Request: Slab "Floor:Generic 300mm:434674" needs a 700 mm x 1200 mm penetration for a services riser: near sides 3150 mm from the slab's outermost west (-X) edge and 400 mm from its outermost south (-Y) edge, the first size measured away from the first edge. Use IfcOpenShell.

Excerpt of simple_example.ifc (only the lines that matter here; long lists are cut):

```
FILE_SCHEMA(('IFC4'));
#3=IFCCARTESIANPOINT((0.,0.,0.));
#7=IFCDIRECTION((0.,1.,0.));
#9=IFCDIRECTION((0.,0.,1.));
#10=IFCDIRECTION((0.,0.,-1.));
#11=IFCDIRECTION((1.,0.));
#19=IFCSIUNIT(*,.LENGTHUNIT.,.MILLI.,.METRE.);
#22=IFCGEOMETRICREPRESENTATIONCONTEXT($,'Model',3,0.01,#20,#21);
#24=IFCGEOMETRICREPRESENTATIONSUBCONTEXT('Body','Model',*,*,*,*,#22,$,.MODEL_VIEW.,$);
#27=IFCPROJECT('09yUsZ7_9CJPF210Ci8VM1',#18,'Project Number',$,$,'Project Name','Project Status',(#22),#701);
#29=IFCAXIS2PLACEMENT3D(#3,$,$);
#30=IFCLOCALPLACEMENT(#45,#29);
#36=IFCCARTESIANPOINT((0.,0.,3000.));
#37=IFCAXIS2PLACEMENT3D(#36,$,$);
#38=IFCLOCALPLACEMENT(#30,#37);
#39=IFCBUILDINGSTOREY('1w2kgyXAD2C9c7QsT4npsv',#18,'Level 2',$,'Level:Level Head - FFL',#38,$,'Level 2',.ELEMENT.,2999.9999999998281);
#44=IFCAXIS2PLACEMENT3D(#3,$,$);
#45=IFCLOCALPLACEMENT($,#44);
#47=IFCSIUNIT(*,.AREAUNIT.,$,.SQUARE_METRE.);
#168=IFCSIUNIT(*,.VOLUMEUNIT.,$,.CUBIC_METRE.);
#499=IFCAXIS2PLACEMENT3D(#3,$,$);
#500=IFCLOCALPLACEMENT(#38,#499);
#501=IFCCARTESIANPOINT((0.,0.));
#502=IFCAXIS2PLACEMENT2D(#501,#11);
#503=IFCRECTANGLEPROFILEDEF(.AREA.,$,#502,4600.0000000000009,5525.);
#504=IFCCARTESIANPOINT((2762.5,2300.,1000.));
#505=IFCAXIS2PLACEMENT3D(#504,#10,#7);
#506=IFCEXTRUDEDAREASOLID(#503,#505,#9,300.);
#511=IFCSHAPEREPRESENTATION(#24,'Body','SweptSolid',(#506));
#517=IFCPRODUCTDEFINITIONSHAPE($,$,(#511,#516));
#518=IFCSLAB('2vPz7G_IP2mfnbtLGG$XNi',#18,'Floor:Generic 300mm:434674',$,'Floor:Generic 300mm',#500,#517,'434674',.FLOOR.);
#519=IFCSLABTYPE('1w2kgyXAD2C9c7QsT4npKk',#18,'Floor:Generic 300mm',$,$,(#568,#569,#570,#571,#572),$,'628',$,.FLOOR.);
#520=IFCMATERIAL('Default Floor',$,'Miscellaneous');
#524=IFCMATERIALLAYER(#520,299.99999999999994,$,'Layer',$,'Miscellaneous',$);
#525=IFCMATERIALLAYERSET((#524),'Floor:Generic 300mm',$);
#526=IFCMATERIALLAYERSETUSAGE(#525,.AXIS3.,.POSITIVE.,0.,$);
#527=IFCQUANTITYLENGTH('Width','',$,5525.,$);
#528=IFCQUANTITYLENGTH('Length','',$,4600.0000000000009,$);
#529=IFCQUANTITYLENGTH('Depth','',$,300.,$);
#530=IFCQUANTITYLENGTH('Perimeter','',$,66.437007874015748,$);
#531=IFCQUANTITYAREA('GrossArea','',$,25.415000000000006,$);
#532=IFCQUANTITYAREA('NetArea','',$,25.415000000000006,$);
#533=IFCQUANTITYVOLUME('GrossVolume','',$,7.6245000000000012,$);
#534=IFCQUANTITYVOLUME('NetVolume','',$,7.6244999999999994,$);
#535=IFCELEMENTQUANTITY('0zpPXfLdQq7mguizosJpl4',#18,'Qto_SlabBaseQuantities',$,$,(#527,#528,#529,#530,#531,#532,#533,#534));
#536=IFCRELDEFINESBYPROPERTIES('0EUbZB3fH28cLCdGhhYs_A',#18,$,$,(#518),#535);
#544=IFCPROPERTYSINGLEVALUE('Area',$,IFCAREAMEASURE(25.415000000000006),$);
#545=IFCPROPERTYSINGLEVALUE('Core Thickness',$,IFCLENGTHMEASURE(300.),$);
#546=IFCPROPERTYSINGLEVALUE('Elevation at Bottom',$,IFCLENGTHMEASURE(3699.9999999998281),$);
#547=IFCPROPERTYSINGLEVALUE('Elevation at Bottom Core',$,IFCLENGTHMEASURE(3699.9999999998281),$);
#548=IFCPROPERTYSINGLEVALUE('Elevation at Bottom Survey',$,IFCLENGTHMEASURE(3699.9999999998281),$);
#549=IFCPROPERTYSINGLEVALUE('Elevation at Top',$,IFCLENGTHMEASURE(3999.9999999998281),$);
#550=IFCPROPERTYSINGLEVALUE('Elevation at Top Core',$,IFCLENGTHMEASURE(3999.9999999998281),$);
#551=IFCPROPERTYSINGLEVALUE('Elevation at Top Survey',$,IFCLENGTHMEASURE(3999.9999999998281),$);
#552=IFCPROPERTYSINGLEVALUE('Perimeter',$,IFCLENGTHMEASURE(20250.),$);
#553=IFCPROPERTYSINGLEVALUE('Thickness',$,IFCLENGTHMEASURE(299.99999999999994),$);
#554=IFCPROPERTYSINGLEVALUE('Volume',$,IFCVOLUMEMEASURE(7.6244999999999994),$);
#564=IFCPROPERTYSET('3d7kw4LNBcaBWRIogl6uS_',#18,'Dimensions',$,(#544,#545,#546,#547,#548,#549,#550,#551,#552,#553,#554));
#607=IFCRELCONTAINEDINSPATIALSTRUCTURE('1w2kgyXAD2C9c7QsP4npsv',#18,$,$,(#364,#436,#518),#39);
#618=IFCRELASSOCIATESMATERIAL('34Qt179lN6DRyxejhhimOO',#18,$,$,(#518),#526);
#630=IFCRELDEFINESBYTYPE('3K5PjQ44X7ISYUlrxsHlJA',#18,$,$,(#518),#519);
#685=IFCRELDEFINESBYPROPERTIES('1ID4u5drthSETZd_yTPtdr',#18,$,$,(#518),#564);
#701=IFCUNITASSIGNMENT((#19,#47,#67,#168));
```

```python
import numpy as np
import ifcopenshell
import ifcopenshell.api.feature
import ifcopenshell.api.geometry
import ifcopenshell.api.pset
import ifcopenshell.api.root
import ifcopenshell.geom
import ifcopenshell.util.element
import ifcopenshell.util.placement
import ifcopenshell.util.representation
import ifcopenshell.util.shape
import ifcopenshell.util.unit

model = ifcopenshell.open("simple_example.ifc")
unit_scale = ifcopenshell.util.unit.calculate_unit_scale(model)
area_scale = ifcopenshell.util.unit.calculate_unit_scale(model, "AREAUNIT")
volume_scale = ifcopenshell.util.unit.calculate_unit_scale(model, "VOLUMEUNIT")
settings = ifcopenshell.geom.settings()


def volume(element):
    """Net volume in cubic metres, openings subtracted."""
    shape = ifcopenshell.geom.create_shape(settings, element)
    return ifcopenshell.util.shape.get_volume(shape.geometry)


slab = model.by_id(518)
before = volume(slab)

# Extent in the slab's own axes, in metres. The edges named are its -X and -Y sides.
slab_shape = ifcopenshell.geom.create_shape(settings, slab)
vertices = ifcopenshell.util.shape.get_vertices(slab_shape.geometry)
x_min, y_min, bottom = vertices.min(axis=0)
top = vertices[:, 2].max()

opening = ifcopenshell.api.root.create_entity(model, ifc_class="IfcOpeningElement", name="Services riser opening", predefined_type="OPENING")
context = ifcopenshell.util.representation.get_context(model, "Model", "Body", "MODEL_VIEW")
width, depth = 0.7, 1.2
outline = [(0.0, 0.0), (width, 0.0), (width, depth), (0.0, depth), (0.0, 0.0)]
# Overshoot both faces by 50 mm so the cut is clean.
shape = ifcopenshell.api.geometry.add_slab_representation(
    model, context=context, depth=top - bottom + 0.1, polyline=outline
)
ifcopenshell.api.geometry.assign_representation(model, product=opening, representation=shape)

matrix = ifcopenshell.util.placement.get_local_placement(slab.ObjectPlacement)
matrix[:, 3] = matrix @ np.append(np.array([x_min + 3.15, y_min + 0.4, bottom - 0.05]) / unit_scale, 1.0)
ifcopenshell.api.geometry.edit_object_placement(model, product=opening, matrix=matrix, is_si=False)
ifcopenshell.api.feature.add_feature(model, feature=opening, element=slab)

after = volume(slab)

# Update the slab's stored quantities.
qto = model.by_id(ifcopenshell.util.element.get_pset(slab, "Qto_SlabBaseQuantities", should_inherit=False)["id"])
ifcopenshell.api.pset.edit_qto(model, qto=qto, properties={
    "NetArea": after / (top - bottom) / area_scale,
    "NetVolume": after / volume_scale,
})
pset = model.by_id(ifcopenshell.util.element.get_pset(slab, "Dimensions", should_inherit=False)["id"])
ifcopenshell.api.pset.edit_pset(model, pset=pset, properties={
    "Area": model.create_entity("IfcAreaMeasure", after / (top - bottom) / area_scale),
    "Volume": model.create_entity("IfcVolumeMeasure", after / volume_scale),
})

print(f"slab volume {before:.3f} -> {after:.3f} m3")

model.write("simple_example_v2.ifc")
```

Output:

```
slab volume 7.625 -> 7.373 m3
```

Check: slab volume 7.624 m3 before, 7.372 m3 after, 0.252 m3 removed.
